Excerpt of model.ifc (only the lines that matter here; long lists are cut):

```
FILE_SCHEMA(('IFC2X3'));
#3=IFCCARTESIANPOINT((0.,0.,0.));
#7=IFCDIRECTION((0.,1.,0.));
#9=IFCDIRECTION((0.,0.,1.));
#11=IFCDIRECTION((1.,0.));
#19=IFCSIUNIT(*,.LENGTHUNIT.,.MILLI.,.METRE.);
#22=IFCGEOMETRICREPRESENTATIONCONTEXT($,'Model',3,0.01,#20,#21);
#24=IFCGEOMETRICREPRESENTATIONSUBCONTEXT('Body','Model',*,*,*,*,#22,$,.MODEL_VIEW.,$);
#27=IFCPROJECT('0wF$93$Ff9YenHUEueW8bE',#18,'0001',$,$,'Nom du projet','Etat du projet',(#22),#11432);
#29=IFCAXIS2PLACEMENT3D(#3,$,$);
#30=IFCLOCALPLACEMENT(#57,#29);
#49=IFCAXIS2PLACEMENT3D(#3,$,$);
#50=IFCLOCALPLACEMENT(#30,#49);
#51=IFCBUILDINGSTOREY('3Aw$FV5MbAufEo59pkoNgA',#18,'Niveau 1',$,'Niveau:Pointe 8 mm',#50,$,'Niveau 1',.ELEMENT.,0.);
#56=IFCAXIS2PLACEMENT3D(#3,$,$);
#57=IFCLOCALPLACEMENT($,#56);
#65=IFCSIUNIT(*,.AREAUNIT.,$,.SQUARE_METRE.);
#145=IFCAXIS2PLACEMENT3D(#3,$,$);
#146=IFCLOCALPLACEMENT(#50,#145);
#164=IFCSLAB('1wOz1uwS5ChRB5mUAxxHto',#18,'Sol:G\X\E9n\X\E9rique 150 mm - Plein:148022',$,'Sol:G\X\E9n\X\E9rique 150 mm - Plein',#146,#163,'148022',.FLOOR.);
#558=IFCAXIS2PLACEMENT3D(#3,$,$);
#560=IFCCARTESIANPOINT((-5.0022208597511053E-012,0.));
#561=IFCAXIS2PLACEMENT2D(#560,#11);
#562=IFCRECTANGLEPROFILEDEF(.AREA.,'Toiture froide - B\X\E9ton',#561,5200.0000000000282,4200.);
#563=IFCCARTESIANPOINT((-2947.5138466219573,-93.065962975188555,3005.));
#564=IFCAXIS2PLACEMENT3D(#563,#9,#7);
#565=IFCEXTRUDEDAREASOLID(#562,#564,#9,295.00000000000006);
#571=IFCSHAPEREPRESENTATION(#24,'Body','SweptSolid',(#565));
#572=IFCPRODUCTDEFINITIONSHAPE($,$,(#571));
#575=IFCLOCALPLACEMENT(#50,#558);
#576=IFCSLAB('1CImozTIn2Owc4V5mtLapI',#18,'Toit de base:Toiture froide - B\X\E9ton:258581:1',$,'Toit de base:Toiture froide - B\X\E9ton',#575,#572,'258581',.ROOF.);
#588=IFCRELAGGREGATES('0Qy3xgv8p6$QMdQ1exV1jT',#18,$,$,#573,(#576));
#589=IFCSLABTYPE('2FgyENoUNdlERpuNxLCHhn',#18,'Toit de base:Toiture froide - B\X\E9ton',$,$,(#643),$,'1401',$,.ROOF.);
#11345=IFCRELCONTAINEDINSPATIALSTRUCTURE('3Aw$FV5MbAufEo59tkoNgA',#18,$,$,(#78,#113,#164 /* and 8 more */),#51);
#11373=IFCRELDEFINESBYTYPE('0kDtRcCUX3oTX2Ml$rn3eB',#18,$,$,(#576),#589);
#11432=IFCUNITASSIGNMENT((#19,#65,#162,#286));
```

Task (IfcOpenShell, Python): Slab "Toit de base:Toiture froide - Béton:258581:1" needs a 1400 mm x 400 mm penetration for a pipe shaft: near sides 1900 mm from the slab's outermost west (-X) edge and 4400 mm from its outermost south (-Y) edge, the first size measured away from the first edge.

```python
import numpy as np
import ifcopenshell
import ifcopenshell.api.feature
import ifcopenshell.api.geometry
import ifcopenshell.api.root
import ifcopenshell.geom
import ifcopenshell.util.placement
import ifcopenshell.util.representation
import ifcopenshell.util.shape
import ifcopenshell.util.unit

model = ifcopenshell.open("model.ifc")
unit_scale = ifcopenshell.util.unit.calculate_unit_scale(model)
settings = ifcopenshell.geom.settings()


def volume(element):
    """Net volume in cubic metres, openings subtracted."""
    shape = ifcopenshell.geom.create_shape(settings, element)
    return ifcopenshell.util.shape.get_volume(shape.geometry)


slab = model.by_guid("1CImozTIn2Owc4V5mtLapI")
before = volume(slab)

# Extent in the slab's own axes, in metres. The edges named are its -X and -Y sides.
slab_shape = ifcopenshell.geom.create_shape(settings, slab)
vertices = ifcopenshell.util.shape.get_vertices(slab_shape.geometry)
x_min, y_min, bottom = vertices.min(axis=0)
top = vertices[:, 2].max()

opening = ifcopenshell.api.root.create_entity(model, ifc_class="IfcOpeningElement", name="Pipe shaft opening")
context = ifcopenshell.util.representation.get_context(model, "Model", "Body", "MODEL_VIEW")
width, depth = 1.4, 0.4
outline = [(0.0, 0.0), (width, 0.0), (width, depth), (0.0, depth), (0.0, 0.0)]
# Overshoot both faces by 50 mm so the cut is clean.
shape = ifcopenshell.api.geometry.add_slab_representation(
    model, context=context, depth=top - bottom + 0.1, polyline=outline
)
ifcopenshell.api.geometry.assign_representation(model, product=opening, representation=shape)

matrix = ifcopenshell.util.placement.get_local_placement(slab.ObjectPlacement)
matrix[:, 3] = matrix @ np.append(np.array([x_min + 1.9, y_min + 4.4, bottom - 0.05]) / unit_scale, 1.0)
ifcopenshell.api.geometry.edit_object_placement(model, product=opening, matrix=matrix, is_si=False)
ifcopenshell.api.feature.add_feature(model, feature=opening, element=slab)

after = volume(slab)

print(f"slab volume {before:.3f} -> {after:.3f} m3")

model.write("model-out.ifc")
```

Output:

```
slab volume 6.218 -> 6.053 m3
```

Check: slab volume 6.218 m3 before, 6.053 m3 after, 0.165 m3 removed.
